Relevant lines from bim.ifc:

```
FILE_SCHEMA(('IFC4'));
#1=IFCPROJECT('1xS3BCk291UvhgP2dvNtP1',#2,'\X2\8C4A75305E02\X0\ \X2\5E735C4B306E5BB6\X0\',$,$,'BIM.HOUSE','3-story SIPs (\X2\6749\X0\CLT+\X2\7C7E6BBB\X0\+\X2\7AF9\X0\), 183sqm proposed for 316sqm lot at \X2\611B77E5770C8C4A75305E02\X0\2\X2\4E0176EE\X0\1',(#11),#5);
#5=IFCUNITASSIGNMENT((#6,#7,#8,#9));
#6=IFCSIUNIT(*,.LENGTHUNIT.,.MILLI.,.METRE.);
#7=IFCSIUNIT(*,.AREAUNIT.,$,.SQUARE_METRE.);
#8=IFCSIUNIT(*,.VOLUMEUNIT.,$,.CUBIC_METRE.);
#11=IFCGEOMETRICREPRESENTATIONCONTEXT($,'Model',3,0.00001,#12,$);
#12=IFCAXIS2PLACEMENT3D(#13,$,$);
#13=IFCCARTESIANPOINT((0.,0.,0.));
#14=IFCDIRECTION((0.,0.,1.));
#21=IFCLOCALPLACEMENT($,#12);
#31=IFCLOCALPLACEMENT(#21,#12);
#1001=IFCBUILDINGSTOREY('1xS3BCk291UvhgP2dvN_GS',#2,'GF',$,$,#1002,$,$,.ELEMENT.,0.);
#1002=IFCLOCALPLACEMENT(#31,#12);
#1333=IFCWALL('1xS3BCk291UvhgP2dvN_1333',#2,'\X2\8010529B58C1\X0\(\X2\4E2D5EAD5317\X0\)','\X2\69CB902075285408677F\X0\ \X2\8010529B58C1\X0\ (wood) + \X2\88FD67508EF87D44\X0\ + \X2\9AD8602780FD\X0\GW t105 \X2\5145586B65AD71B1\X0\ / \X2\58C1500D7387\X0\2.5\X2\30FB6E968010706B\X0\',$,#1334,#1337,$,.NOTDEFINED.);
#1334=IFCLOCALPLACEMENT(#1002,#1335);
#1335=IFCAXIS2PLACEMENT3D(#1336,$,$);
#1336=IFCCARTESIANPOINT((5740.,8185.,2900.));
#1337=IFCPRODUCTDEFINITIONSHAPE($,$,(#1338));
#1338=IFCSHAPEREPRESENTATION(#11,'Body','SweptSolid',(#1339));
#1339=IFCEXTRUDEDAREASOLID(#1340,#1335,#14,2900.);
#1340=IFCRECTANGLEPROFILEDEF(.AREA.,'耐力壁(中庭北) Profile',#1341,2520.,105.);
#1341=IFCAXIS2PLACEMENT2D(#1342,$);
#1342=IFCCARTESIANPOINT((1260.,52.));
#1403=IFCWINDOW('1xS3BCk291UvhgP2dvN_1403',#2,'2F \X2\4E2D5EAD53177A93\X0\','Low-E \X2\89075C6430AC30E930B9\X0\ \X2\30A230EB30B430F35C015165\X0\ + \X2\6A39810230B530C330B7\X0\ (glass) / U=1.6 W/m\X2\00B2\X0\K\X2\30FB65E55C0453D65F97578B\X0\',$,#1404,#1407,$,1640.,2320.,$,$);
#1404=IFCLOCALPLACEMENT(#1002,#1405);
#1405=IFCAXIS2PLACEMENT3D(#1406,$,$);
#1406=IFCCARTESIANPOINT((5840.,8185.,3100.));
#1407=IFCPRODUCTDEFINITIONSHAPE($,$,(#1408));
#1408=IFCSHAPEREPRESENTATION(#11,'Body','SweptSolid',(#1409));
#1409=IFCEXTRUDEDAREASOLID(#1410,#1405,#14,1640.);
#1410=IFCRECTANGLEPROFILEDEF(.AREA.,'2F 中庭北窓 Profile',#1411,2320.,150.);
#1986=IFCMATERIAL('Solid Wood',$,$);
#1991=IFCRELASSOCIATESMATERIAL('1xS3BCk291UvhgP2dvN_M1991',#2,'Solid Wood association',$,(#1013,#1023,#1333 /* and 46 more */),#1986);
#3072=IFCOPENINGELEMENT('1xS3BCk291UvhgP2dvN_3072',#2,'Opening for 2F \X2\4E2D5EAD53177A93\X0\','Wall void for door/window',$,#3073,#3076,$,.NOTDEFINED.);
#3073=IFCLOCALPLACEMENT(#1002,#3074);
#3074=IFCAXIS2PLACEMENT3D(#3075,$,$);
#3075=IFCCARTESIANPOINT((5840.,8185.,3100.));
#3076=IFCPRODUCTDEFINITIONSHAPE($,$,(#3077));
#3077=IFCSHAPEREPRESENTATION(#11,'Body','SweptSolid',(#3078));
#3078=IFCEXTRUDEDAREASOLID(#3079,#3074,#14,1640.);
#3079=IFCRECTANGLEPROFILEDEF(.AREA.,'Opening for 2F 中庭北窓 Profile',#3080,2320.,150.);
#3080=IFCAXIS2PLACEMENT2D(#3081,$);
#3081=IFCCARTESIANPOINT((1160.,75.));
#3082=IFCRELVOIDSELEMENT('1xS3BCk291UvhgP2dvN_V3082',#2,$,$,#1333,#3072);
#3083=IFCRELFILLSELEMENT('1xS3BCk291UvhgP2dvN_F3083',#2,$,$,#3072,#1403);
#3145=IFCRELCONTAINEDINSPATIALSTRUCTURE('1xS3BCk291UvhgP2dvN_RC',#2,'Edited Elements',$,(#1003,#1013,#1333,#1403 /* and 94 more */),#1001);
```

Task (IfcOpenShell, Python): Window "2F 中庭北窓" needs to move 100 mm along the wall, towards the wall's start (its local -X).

```python
import ifcopenshell
import ifcopenshell.api.geometry
import ifcopenshell.util.placement

model = ifcopenshell.open("bim.ifc")

window = model.by_guid("1xS3BCk291UvhgP2dvN_1403")
opening = window.FillsVoids[0].RelatingOpeningElement
wall = opening.VoidsElements[0].RelatingBuildingElement

wall_matrix = ifcopenshell.util.placement.get_local_placement(wall.ObjectPlacement)
shift = wall_matrix[:3, 0] * -100.0
before = ifcopenshell.util.placement.get_local_placement(window.ObjectPlacement)[:3, 3].copy()

# The window is not placed relative to its opening, so move both.
for product in (opening, window):
    matrix = ifcopenshell.util.placement.get_local_placement(product.ObjectPlacement)
    matrix[:3, 3] += shift
    ifcopenshell.api.geometry.edit_object_placement(model, product=product, matrix=matrix, is_si=False)

after = ifcopenshell.util.placement.get_local_placement(window.ObjectPlacement)[:3, 3]
print("window moved by", (after - before).round(3) + 0.0)

model.write("bim_rev.ifc")
```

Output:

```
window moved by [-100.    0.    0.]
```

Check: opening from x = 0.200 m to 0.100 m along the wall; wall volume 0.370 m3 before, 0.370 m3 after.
